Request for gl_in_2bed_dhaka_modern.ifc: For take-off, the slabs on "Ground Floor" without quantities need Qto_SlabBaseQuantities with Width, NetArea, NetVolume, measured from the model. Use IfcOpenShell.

First a look at what the model holds.

```python
import ifcopenshell
import ifcopenshell.util.element
import ifcopenshell.util.unit

model = ifcopenshell.open("gl_in_2bed_dhaka_modern.ifc")
print(model.schema)
for unit_type in ("LENGTHUNIT", "AREAUNIT", "VOLUMEUNIT"):
    print(unit_type, ifcopenshell.util.unit.calculate_unit_scale(model, unit_type))
storey = next(s for s in model.by_type("IfcBuildingStorey") if s.Name == "Ground Floor")
slabs = [e for e in ifcopenshell.util.element.get_decomposition(storey) if e.is_a("IfcSlab")]
for e in sorted(slabs, key=lambda e: e.id()):
    print(e.id(), e.is_a(), e.Name, list(ifcopenshell.util.element.get_psets(e, qtos_only=True)), sep=" | ")
```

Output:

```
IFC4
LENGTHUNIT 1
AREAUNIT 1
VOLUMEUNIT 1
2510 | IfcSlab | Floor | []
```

```python
import ifcopenshell
import ifcopenshell.api.pset
import ifcopenshell.geom
import ifcopenshell.util.element
import ifcopenshell.util.shape
import ifcopenshell.util.unit

model = ifcopenshell.open("gl_in_2bed_dhaka_modern.ifc")
unit_scale = ifcopenshell.util.unit.calculate_unit_scale(model)
area_scale = ifcopenshell.util.unit.calculate_unit_scale(model, "AREAUNIT")
volume_scale = ifcopenshell.util.unit.calculate_unit_scale(model, "VOLUMEUNIT")
settings = ifcopenshell.geom.settings()

storey = next(s for s in model.by_type("IfcBuildingStorey") if s.Name == "Ground Floor")
slabs = [e for e in ifcopenshell.util.element.get_decomposition(storey) if e.is_a("IfcSlab")]

for e in sorted(slabs, key=lambda e: e.id()):
    if ifcopenshell.util.element.get_psets(e, qtos_only=True, should_inherit=False):
        continue
    # Geometry comes back in metres, in the element's own axes.
    shape = ifcopenshell.geom.create_shape(settings, e)
    values = {
        "Width": ifcopenshell.util.shape.get_z(shape.geometry) / unit_scale,
        "NetArea": ifcopenshell.util.shape.get_footprint_area(shape.geometry) / area_scale,
        "NetVolume": ifcopenshell.util.shape.get_volume(shape.geometry) / volume_scale,
    }
    qto = ifcopenshell.api.pset.add_qto(model, product=e, name="Qto_SlabBaseQuantities")
    ifcopenshell.api.pset.edit_qto(model, qto=qto, properties=values)
    print(e.id(), {k: round(v, 3) for k, v in values.items()})

model.write("gl_in_2bed_dhaka_modern_edited.ifc")
```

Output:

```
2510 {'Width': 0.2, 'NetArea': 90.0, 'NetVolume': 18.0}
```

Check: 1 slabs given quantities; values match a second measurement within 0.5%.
